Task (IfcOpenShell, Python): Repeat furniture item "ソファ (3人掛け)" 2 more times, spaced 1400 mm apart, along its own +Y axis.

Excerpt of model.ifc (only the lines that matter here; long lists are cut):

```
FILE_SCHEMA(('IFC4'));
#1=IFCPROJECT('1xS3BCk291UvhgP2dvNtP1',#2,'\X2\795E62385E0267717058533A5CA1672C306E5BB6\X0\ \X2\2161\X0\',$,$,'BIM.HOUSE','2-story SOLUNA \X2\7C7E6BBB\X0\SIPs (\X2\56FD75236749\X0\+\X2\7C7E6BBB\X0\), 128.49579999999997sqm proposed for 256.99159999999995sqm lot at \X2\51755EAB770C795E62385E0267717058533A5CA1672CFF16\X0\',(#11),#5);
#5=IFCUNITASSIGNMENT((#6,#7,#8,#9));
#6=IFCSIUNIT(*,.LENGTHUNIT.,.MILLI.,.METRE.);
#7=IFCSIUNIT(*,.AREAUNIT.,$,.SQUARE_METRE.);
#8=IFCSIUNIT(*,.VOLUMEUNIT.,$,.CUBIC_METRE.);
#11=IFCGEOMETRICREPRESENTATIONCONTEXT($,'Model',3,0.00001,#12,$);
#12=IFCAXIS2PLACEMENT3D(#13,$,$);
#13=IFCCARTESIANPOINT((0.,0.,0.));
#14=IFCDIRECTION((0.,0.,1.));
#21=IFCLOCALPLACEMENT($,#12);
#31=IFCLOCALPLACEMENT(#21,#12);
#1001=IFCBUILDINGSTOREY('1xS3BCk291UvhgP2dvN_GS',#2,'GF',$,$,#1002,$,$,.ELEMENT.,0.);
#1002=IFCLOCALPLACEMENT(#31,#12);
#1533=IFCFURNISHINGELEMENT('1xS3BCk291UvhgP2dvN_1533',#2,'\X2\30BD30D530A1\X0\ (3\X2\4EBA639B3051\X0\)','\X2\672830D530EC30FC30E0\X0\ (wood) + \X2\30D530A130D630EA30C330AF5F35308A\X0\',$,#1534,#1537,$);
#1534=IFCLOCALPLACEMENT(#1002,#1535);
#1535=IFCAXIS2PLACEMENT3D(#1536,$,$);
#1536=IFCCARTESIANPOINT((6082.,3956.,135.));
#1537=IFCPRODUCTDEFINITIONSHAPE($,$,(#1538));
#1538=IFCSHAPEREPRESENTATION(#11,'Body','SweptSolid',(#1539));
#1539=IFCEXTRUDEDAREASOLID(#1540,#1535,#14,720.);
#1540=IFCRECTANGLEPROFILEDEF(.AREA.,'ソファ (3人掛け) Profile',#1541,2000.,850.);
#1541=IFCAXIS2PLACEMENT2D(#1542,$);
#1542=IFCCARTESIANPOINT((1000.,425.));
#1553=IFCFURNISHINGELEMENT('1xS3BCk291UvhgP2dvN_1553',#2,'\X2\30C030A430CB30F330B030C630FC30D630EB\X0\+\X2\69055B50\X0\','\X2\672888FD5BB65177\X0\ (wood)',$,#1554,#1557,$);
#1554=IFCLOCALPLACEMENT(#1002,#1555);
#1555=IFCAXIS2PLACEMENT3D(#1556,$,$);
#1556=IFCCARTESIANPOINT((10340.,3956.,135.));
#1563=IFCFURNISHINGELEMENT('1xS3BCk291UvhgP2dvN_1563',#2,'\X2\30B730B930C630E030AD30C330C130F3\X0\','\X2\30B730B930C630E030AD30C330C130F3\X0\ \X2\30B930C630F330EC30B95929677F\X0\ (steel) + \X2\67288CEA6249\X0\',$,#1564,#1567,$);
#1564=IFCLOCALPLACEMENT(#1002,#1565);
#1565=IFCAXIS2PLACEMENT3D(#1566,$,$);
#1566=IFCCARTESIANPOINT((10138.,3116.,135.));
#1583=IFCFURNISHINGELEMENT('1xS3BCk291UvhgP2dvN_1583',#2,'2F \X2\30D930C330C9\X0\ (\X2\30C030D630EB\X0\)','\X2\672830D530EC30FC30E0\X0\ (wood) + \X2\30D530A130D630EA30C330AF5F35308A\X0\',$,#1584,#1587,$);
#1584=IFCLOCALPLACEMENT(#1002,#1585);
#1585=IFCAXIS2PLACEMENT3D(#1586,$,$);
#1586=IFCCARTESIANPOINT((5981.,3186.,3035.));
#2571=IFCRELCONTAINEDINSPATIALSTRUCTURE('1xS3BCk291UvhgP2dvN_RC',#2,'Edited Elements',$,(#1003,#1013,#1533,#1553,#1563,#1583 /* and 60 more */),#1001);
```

```python
import ifcopenshell
import ifcopenshell.api.geometry
import ifcopenshell.api.root
import ifcopenshell.util.element
import ifcopenshell.util.placement
import ifcopenshell.util.unit

model = ifcopenshell.open("model.ifc")
unit_scale = ifcopenshell.util.unit.calculate_unit_scale(model)


def reuse_history(source, copy):
    """copy_class also copies each property set's owner history, people and application; keep the originals."""
    for rel in copy.IsDefinedBy:
        if rel.is_a("IfcRelDefinesByProperties") and (history := rel.RelatingPropertyDefinition.OwnerHistory):
            rel.RelatingPropertyDefinition.OwnerHistory = source.OwnerHistory
            ifcopenshell.util.element.remove_deep2(model, history)


source = model.by_id(1533)
base = ifcopenshell.util.placement.get_local_placement(source.ObjectPlacement)
step = base[:3, 1] * 1.4 / unit_scale

for i in range(1, 3):
    copy = ifcopenshell.api.root.copy_class(model, product=source)
    copy.Representation = ifcopenshell.util.element.copy_deep(
        model, source.Representation, exclude=["IfcGeometricRepresentationContext", "IfcRepresentationMap"]
    )
    reuse_history(source, copy)
    matrix = base.copy()
    matrix[:3, 3] += i * step
    print("added at", matrix[:3, 3].round(3) + 0.0)
    ifcopenshell.api.geometry.edit_object_placement(model, product=copy, matrix=matrix, is_si=False)

model.write("model_edited.ifc")
```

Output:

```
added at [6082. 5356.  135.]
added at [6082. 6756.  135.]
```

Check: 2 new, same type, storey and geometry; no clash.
